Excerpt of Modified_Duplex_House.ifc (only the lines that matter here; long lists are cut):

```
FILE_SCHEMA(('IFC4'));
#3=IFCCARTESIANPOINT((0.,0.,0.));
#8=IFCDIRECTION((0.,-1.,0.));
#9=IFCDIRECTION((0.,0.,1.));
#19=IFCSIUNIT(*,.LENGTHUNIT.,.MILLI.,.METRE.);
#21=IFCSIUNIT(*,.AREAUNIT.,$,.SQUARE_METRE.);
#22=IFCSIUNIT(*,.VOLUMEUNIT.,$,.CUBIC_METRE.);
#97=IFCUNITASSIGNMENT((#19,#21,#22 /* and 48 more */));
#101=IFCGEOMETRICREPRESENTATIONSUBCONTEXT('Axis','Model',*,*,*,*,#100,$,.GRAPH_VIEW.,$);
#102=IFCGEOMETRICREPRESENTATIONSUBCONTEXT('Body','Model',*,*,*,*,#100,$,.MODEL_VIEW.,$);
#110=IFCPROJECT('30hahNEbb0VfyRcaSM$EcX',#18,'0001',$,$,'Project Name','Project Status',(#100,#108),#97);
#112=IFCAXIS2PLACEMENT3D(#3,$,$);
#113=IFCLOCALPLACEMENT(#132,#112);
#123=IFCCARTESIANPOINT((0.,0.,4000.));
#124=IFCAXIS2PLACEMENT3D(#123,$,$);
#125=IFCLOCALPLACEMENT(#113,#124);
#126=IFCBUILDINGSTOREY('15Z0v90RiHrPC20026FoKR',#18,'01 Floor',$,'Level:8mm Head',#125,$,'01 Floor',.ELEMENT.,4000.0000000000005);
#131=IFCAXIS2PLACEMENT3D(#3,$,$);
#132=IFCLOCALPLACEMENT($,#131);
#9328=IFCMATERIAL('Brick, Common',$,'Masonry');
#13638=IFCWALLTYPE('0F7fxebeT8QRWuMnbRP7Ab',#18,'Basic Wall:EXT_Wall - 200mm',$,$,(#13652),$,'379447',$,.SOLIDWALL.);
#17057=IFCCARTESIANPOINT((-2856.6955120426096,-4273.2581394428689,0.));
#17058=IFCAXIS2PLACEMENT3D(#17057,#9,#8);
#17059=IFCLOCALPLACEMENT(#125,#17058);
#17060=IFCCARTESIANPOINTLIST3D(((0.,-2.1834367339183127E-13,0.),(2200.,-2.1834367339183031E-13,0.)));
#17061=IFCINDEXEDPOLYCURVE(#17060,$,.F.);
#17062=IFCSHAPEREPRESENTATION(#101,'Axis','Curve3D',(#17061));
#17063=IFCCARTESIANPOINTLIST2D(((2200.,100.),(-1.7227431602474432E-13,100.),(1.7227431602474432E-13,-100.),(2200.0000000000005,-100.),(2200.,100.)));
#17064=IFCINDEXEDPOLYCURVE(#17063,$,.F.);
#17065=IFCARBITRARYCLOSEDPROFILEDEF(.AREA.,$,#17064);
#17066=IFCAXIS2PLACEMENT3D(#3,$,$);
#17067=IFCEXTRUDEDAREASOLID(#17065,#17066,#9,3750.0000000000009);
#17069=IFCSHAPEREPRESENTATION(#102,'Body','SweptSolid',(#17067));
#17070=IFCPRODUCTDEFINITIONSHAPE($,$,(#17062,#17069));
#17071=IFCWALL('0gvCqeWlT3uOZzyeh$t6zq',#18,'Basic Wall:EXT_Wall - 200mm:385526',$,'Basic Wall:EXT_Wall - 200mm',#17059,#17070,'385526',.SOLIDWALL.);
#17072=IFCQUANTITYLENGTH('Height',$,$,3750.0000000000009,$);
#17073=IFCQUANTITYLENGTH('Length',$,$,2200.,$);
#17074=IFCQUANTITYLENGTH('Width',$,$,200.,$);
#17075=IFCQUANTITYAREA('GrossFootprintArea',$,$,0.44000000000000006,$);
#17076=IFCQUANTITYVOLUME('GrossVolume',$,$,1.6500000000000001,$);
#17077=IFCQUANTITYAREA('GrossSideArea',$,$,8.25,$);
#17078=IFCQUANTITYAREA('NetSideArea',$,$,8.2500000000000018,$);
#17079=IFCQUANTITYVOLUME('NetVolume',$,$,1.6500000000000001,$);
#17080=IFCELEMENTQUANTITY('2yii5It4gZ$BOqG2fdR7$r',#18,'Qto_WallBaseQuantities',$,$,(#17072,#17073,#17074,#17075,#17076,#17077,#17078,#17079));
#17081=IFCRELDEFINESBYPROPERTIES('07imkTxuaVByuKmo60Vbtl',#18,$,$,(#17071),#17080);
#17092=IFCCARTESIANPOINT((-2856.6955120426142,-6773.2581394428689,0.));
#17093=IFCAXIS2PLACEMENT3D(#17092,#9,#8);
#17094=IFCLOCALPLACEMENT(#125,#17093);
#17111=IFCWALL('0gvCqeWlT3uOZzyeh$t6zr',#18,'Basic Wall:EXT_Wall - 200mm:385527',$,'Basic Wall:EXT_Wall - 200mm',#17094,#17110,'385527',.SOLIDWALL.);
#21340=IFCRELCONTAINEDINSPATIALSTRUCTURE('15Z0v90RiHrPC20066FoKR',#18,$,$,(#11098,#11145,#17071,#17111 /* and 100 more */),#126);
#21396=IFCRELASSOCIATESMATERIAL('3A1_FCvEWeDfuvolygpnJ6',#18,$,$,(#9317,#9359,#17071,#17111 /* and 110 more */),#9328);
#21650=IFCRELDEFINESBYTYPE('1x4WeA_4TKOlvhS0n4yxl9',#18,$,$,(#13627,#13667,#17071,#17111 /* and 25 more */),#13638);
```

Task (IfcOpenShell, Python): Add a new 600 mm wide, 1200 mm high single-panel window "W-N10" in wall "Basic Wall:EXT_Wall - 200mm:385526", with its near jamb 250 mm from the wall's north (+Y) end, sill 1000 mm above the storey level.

```python
import numpy as np
import ifcopenshell
import ifcopenshell.api.feature
import ifcopenshell.api.geometry
import ifcopenshell.api.pset
import ifcopenshell.api.root
import ifcopenshell.api.spatial
import ifcopenshell.geom
import ifcopenshell.util.element
import ifcopenshell.util.placement
import ifcopenshell.util.representation
import ifcopenshell.util.shape
import ifcopenshell.util.unit

model = ifcopenshell.open("Modified_Duplex_House.ifc")
unit_scale = ifcopenshell.util.unit.calculate_unit_scale(model)
area_scale = ifcopenshell.util.unit.calculate_unit_scale(model, "AREAUNIT")
volume_scale = ifcopenshell.util.unit.calculate_unit_scale(model, "VOLUMEUNIT")
settings = ifcopenshell.geom.settings()


def volume(element):
    """Net volume in cubic metres, openings subtracted."""
    shape = ifcopenshell.geom.create_shape(settings, element)
    return ifcopenshell.util.shape.get_volume(shape.geometry)


wall = model.by_guid("0gvCqeWlT3uOZzyeh$t6zq")
storey = ifcopenshell.util.element.get_container(wall, ifc_class="IfcBuildingStorey")
context = ifcopenshell.util.representation.get_context(model, "Model", "Body", "MODEL_VIEW")
before = volume(wall)

width, height, from_end, sill = 0.6, 1.2, 0.25, 1  # metres

# The wall runs along its own X axis, and the end named is its -X end.
wall_shape = ifcopenshell.geom.create_shape(settings, wall)
x, y, z = ifcopenshell.util.shape.get_vertices(wall_shape.geometry).T
start = x.min() + from_end
face, thickness = float(y.min()), float(y.max() - y.min())
wall_matrix = ifcopenshell.util.placement.get_local_placement(wall.ObjectPlacement)
level = ifcopenshell.util.placement.get_local_placement(storey.ObjectPlacement)[2, 3]


def in_wall(x, y):
    """Placement at x, y metres in the wall's axes, at sill height."""
    matrix = wall_matrix.copy()
    matrix[:, 3] = wall_matrix @ np.array([x / unit_scale, y / unit_scale, 0.0, 1.0])
    matrix[2, 3] = level + sill / unit_scale
    return matrix


# Opening: a box that overshoots both wall faces by 50 mm.
opening = ifcopenshell.api.root.create_entity(model, ifc_class="IfcOpeningElement", predefined_type="OPENING")
box = ifcopenshell.api.geometry.add_wall_representation(
    model, context=context, length=width, height=height, thickness=thickness + 0.1
)
ifcopenshell.api.geometry.assign_representation(model, product=opening, representation=box)
ifcopenshell.api.geometry.edit_object_placement(model, product=opening, matrix=in_wall(start, face - 0.05), is_si=False)
ifcopenshell.api.feature.add_feature(model, feature=opening, element=wall)

window = ifcopenshell.api.root.create_entity(model, ifc_class="IfcWindow", name="W-N10", predefined_type="WINDOW")
window.OverallWidth, window.OverallHeight = width / unit_scale, height / unit_scale
window.PartitioningType = "SINGLE_PANEL"
body = ifcopenshell.api.geometry.add_window_representation(
    model,
    context=context,
    overall_width=window.OverallWidth,
    overall_height=window.OverallHeight,
    partition_type="SINGLE_PANEL",
)
ifcopenshell.api.geometry.assign_representation(model, product=window, representation=body)
ifcopenshell.api.spatial.assign_container(model, products=[window], relating_structure=storey)
ifcopenshell.api.feature.add_filling(model, opening=opening, element=window)

# Centre the window in the wall's thickness.
ifcopenshell.api.geometry.edit_object_placement(model, product=window, matrix=in_wall(start, face), is_si=False)
window_shape = ifcopenshell.geom.create_shape(settings, window)
depth = ifcopenshell.util.shape.get_vertices(window_shape.geometry)[:, 1]
offset = face + thickness / 2 - (depth.min() + depth.max()) / 2
ifcopenshell.api.geometry.edit_object_placement(model, product=window, matrix=in_wall(start, offset), is_si=False)

after = volume(wall)

# Update the wall's stored quantities.
qto = model.by_id(ifcopenshell.util.element.get_pset(wall, "Qto_WallBaseQuantities", should_inherit=False)["id"])
ifcopenshell.api.pset.edit_qto(model, qto=qto, properties={
    "NetSideArea": after / thickness / area_scale,
    "NetVolume": after / volume_scale,
})

print(f"wall volume {before:.3f} -> {after:.3f} m3")

model.write("Modified_Duplex_House_updated.ifc")
```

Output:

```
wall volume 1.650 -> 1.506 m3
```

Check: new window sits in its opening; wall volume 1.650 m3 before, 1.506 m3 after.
